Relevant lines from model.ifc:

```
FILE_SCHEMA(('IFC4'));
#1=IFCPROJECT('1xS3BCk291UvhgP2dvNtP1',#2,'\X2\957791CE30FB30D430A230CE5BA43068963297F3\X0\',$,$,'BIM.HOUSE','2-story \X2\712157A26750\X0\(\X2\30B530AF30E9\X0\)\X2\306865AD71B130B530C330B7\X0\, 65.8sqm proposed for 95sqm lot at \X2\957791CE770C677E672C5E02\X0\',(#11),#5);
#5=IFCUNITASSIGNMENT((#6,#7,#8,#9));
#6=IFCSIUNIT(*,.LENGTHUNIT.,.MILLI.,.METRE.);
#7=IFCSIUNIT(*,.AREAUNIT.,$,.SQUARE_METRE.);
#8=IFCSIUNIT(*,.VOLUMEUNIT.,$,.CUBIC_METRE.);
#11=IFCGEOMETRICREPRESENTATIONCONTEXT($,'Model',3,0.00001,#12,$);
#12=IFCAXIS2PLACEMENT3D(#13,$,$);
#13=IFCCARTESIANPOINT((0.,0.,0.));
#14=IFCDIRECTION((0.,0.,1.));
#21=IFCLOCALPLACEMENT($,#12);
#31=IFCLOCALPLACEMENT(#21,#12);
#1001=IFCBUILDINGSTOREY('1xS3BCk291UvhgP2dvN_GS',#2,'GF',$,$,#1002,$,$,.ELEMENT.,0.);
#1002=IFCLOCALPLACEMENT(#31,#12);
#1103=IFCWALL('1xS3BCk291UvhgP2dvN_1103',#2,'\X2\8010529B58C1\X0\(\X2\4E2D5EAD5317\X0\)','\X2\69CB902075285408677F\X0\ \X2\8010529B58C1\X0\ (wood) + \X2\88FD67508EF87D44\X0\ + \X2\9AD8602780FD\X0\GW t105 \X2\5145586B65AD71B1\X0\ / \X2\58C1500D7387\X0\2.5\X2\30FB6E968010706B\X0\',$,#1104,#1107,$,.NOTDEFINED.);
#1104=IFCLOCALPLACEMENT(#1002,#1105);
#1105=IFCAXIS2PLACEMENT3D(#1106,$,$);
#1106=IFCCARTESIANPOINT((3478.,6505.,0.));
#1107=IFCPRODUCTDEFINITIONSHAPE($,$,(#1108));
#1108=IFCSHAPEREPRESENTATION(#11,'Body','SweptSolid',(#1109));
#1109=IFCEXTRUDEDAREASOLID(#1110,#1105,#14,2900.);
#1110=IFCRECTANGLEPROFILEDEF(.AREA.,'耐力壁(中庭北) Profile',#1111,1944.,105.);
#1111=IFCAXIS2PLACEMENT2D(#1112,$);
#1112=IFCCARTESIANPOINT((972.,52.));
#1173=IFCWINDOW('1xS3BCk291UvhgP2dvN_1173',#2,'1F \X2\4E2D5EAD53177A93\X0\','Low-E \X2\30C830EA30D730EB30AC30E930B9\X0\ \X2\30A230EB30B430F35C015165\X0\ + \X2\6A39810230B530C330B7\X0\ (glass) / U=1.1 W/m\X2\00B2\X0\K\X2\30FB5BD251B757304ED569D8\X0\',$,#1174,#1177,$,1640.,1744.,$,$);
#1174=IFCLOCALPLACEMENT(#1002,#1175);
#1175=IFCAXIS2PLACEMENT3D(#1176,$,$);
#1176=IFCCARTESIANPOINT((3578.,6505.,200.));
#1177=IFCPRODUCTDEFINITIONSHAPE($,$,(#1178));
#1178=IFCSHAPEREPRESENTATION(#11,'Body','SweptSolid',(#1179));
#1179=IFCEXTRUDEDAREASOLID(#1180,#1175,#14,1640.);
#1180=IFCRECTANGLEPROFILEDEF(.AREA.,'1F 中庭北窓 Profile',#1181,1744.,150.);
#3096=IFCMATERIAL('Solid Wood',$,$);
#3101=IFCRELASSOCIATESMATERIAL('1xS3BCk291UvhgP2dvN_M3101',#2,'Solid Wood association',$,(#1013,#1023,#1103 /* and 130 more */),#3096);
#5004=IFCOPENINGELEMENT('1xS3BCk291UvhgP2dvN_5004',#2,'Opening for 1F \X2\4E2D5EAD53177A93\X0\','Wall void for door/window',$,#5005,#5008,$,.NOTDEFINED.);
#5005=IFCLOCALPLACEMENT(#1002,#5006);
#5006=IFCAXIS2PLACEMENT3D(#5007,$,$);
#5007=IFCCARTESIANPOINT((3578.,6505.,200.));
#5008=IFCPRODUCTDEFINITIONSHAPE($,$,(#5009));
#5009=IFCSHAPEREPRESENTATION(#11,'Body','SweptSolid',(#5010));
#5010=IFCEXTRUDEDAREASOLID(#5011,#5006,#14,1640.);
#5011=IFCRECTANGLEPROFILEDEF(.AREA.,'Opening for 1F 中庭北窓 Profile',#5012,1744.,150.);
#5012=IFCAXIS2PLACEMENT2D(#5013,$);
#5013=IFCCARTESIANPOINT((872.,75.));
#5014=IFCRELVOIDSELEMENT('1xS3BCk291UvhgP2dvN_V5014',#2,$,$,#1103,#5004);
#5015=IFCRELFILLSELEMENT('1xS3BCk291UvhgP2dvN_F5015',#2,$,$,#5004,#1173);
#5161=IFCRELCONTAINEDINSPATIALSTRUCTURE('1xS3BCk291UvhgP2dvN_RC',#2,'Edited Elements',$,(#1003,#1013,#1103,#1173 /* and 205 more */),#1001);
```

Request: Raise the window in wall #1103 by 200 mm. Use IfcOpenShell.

```python
import numpy as np
import ifcopenshell
import ifcopenshell.api.geometry
import ifcopenshell.util.placement
import ifcopenshell.util.unit

model = ifcopenshell.open("model.ifc")
unit_scale = ifcopenshell.util.unit.calculate_unit_scale(model)

window = model.by_id(1173)
opening = window.FillsVoids[0].RelatingOpeningElement
dz = 0.2 / unit_scale

shift = np.array([0.0, 0.0, dz])
# The window is not placed relative to its opening, so move both.
for product in (opening, window):
    matrix = ifcopenshell.util.placement.get_local_placement(product.ObjectPlacement)
    matrix[:3, 3] += shift
    ifcopenshell.api.geometry.edit_object_placement(model, product=product, matrix=matrix, is_si=False)

print(f"moved by {dz * unit_scale:+.3f} m")

model.write("model-out.ifc")
```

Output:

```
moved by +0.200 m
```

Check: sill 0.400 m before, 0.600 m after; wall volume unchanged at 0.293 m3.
